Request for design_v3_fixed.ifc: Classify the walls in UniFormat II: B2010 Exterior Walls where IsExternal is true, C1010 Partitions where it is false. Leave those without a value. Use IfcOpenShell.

First a look at what the model holds.

```python
import ifcopenshell
import ifcopenshell.util.element

model = ifcopenshell.open("design_v3_fixed.ifc")
print(model.schema)
print("classifications:", [c.Name for c in model.by_type("IfcClassification")])
values = [ifcopenshell.util.element.get_pset(e, "Pset_WallCommon", "IsExternal") for e in model.by_type("IfcWall")]
for value in (True, False, None):
    print("IsExternal", value, values.count(value))
```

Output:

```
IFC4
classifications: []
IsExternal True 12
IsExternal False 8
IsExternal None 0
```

```python
import ifcopenshell
import ifcopenshell.api.classification
import ifcopenshell.util.element

model = ifcopenshell.open("design_v3_fixed.ifc")

system = ifcopenshell.api.classification.add_classification(model, classification="UniFormat II")

walls = model.by_type("IfcWall")
external = {e: ifcopenshell.util.element.get_pset(e, "Pset_WallCommon", "IsExternal") for e in walls}
for flag, code, name in ((True, "B2010", "Exterior Walls"), (False, "C1010", "Partitions")):
    products = [e for e in walls if external[e] is flag]
    ifcopenshell.api.classification.add_reference(
        model, products=products, classification=system, identification=code, name=name
    )
    print(code, len(products))

model.write("design_v3_fixed_edited.ifc")
```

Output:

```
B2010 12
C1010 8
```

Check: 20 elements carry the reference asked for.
